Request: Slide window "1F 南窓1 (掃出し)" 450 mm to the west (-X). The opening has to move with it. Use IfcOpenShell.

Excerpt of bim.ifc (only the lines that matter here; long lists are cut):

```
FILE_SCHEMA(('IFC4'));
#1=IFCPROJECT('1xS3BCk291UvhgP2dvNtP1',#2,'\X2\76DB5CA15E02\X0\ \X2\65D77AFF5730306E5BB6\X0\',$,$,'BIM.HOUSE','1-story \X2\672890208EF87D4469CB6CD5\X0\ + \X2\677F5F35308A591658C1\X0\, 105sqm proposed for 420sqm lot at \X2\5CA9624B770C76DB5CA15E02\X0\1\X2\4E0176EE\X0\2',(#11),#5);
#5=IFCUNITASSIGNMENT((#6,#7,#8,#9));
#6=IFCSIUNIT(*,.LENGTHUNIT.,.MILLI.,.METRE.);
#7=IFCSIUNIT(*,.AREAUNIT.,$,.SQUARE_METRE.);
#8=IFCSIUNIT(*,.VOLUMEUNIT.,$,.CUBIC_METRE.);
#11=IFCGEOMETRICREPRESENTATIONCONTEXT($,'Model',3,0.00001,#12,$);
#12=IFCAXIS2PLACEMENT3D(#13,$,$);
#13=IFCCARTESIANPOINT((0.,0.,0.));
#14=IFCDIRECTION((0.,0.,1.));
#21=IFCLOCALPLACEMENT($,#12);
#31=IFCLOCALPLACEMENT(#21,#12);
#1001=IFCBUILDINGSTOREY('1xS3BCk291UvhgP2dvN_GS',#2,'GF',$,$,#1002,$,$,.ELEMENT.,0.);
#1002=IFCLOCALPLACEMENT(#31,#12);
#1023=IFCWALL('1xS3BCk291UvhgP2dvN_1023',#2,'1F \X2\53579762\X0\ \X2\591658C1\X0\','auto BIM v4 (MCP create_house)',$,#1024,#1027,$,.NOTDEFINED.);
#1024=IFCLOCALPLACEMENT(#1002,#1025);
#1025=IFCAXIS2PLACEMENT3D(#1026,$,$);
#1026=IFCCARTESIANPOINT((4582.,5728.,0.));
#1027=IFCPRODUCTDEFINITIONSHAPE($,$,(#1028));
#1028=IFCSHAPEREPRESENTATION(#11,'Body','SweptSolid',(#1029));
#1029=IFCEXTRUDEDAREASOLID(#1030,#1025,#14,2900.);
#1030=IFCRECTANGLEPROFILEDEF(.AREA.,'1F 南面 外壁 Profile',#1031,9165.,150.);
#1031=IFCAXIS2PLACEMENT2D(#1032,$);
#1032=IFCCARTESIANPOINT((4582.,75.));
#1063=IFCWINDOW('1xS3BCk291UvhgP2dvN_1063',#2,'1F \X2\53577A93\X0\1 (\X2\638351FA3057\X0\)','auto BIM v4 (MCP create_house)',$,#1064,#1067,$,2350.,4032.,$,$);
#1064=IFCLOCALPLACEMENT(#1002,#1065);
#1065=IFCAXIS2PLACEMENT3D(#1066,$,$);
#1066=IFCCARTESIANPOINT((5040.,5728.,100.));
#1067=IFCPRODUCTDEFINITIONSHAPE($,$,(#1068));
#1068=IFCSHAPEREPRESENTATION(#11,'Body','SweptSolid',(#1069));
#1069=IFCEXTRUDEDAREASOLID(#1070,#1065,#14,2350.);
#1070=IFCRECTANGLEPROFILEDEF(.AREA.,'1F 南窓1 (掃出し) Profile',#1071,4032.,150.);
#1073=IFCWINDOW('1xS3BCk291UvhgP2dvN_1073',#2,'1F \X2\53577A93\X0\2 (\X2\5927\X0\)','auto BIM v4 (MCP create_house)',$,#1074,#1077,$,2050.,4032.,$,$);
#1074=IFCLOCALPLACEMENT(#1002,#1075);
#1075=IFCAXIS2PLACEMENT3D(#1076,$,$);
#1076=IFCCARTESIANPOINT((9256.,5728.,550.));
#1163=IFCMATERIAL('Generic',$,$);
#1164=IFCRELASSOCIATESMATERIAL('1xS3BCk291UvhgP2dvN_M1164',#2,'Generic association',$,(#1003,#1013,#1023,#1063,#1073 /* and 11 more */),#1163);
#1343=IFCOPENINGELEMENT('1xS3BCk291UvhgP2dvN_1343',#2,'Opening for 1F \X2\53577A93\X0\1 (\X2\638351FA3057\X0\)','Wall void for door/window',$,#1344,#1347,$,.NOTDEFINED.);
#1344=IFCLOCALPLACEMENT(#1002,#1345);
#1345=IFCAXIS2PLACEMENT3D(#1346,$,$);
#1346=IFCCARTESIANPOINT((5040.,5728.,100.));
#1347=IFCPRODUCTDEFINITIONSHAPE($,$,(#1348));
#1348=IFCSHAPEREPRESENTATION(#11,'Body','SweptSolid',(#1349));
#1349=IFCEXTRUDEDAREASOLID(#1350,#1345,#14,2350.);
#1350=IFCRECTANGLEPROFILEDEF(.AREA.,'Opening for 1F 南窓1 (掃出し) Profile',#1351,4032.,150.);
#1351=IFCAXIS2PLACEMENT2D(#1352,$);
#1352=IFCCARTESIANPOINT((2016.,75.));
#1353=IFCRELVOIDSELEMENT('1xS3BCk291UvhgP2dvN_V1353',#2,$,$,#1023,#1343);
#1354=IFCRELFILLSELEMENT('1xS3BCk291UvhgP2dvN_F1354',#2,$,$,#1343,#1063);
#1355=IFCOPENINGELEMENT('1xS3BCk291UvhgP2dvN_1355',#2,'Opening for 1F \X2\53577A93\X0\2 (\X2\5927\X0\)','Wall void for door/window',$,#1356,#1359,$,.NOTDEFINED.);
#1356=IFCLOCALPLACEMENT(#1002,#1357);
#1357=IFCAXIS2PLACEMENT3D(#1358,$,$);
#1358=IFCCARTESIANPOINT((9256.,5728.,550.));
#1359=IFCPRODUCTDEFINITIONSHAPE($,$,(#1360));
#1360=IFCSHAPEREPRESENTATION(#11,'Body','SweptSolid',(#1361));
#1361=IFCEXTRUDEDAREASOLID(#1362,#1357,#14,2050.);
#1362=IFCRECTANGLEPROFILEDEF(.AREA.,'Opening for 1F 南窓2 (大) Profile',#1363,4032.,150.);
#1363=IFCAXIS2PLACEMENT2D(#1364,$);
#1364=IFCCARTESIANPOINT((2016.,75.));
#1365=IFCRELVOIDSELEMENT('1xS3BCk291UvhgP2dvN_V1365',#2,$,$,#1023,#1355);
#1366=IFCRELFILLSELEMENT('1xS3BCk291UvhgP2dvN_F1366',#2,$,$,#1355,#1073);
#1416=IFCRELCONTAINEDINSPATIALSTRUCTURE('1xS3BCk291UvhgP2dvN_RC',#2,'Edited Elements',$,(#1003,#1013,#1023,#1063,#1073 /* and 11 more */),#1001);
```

```python
import ifcopenshell
import ifcopenshell.api.geometry
import ifcopenshell.util.placement
import ifcopenshell.util.unit

model = ifcopenshell.open("bim.ifc")
unit_scale = ifcopenshell.util.unit.calculate_unit_scale(model)

window = model.by_guid("1xS3BCk291UvhgP2dvN_1063")
opening = window.FillsVoids[0].RelatingOpeningElement
wall = opening.VoidsElements[0].RelatingBuildingElement

wall_matrix = ifcopenshell.util.placement.get_local_placement(wall.ObjectPlacement)
shift = wall_matrix[:3, 0] * -0.45 / unit_scale
before = ifcopenshell.util.placement.get_local_placement(window.ObjectPlacement)[:3, 3].copy()

# The window is not placed relative to its opening, so move both.
for product in (opening, window):
    matrix = ifcopenshell.util.placement.get_local_placement(product.ObjectPlacement)
    matrix[:3, 3] += shift
    ifcopenshell.api.geometry.edit_object_placement(model, product=product, matrix=matrix, is_si=False)

after = ifcopenshell.util.placement.get_local_placement(window.ObjectPlacement)[:3, 3]
print("window moved by", (after - before).round(3) + 0.0)

model.write("bim_updated.ifc")
```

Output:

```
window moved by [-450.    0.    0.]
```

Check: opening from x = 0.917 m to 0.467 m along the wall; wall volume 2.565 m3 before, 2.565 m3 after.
